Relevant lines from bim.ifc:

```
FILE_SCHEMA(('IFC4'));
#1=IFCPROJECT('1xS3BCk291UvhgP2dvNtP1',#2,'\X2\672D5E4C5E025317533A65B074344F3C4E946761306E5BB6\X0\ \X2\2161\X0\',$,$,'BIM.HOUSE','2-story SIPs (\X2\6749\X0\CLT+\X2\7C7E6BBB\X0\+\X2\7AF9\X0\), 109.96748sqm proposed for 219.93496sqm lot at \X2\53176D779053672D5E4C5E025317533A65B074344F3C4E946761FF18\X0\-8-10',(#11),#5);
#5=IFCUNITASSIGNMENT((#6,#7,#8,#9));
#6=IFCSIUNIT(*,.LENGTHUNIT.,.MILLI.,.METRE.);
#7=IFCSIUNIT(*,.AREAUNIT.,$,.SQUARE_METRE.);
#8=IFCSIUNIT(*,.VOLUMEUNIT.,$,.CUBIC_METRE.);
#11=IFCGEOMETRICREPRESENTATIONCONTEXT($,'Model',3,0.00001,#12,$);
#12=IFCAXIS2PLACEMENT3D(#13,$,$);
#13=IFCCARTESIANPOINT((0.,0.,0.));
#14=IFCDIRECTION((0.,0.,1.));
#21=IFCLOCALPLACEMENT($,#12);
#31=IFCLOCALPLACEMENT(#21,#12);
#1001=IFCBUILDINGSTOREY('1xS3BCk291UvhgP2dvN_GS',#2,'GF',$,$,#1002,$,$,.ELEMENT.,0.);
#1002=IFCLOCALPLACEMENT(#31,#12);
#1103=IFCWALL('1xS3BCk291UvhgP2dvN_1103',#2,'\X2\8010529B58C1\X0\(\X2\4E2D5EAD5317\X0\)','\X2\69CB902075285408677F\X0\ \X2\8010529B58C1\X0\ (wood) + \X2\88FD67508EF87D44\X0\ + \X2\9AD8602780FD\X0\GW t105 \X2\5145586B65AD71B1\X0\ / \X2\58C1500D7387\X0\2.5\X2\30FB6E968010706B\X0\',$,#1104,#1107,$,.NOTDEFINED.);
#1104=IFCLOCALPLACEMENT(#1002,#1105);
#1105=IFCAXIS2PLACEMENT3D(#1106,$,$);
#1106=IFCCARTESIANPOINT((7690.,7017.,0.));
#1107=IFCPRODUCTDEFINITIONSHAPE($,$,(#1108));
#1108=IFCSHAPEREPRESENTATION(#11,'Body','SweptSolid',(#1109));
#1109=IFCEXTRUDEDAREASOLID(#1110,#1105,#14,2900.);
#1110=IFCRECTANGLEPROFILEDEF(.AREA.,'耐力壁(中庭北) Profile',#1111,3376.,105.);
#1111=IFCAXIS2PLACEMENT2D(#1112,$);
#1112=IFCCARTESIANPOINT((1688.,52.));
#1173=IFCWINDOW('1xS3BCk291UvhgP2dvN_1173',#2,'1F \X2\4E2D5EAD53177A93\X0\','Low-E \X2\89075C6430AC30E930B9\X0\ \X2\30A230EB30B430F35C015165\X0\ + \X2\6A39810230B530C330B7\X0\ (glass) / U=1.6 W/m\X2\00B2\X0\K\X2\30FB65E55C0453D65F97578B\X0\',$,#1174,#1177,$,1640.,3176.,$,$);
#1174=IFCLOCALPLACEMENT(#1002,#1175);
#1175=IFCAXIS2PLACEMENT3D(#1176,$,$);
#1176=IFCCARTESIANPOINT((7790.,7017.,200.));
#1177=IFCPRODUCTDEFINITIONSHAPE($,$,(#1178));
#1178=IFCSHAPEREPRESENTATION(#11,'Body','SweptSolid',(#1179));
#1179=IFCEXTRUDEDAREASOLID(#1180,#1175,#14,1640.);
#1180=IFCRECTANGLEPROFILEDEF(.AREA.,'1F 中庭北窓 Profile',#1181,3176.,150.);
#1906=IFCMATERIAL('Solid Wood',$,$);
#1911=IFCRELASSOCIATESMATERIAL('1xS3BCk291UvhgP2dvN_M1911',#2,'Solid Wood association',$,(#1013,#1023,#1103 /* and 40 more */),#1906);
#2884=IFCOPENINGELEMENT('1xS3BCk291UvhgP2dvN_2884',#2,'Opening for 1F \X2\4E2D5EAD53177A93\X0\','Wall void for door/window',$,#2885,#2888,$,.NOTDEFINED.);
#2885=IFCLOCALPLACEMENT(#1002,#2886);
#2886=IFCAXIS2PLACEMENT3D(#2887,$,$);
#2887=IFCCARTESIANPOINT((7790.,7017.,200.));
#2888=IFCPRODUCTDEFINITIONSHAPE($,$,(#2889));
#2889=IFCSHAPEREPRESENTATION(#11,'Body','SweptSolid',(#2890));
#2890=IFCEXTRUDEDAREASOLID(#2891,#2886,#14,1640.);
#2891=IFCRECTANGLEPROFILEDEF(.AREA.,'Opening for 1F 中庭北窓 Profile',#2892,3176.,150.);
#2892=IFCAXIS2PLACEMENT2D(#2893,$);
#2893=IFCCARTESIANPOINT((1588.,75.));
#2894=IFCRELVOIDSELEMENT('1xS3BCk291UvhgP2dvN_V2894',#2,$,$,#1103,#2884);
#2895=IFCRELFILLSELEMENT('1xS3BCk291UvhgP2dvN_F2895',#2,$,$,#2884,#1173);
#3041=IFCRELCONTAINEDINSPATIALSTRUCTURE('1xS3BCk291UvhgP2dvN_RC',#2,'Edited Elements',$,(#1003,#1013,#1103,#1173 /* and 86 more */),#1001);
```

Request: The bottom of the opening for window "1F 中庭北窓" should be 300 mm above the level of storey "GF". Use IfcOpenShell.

```python
import numpy as np
import ifcopenshell
import ifcopenshell.api.geometry
import ifcopenshell.geom
import ifcopenshell.util.element
import ifcopenshell.util.placement
import ifcopenshell.util.shape
import ifcopenshell.util.unit

model = ifcopenshell.open("bim.ifc")
unit_scale = ifcopenshell.util.unit.calculate_unit_scale(model)

window = model.by_guid("1xS3BCk291UvhgP2dvN_1173")
opening = window.FillsVoids[0].RelatingOpeningElement
storey = ifcopenshell.util.element.get_container(window, ifc_class="IfcBuildingStorey")
level = ifcopenshell.util.placement.get_local_placement(storey.ObjectPlacement)[2, 3]

# The opening's origin need not be at the sill, so measure its lowest point.
shape = ifcopenshell.geom.create_shape(ifcopenshell.geom.settings(), opening)
bottom = ifcopenshell.util.shape.get_shape_bottom_elevation(shape, shape.geometry) / unit_scale
dz = level + 0.3 / unit_scale - bottom

shift = np.array([0.0, 0.0, dz])
# The window is not placed relative to its opening, so move both.
for product in (opening, window):
    matrix = ifcopenshell.util.placement.get_local_placement(product.ObjectPlacement)
    matrix[:3, 3] += shift
    ifcopenshell.api.geometry.edit_object_placement(model, product=product, matrix=matrix, is_si=False)

print(f"moved by {dz * unit_scale:+.3f} m")

model.write("bim-out.ifc")
```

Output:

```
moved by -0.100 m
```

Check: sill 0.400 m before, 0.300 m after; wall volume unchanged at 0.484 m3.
